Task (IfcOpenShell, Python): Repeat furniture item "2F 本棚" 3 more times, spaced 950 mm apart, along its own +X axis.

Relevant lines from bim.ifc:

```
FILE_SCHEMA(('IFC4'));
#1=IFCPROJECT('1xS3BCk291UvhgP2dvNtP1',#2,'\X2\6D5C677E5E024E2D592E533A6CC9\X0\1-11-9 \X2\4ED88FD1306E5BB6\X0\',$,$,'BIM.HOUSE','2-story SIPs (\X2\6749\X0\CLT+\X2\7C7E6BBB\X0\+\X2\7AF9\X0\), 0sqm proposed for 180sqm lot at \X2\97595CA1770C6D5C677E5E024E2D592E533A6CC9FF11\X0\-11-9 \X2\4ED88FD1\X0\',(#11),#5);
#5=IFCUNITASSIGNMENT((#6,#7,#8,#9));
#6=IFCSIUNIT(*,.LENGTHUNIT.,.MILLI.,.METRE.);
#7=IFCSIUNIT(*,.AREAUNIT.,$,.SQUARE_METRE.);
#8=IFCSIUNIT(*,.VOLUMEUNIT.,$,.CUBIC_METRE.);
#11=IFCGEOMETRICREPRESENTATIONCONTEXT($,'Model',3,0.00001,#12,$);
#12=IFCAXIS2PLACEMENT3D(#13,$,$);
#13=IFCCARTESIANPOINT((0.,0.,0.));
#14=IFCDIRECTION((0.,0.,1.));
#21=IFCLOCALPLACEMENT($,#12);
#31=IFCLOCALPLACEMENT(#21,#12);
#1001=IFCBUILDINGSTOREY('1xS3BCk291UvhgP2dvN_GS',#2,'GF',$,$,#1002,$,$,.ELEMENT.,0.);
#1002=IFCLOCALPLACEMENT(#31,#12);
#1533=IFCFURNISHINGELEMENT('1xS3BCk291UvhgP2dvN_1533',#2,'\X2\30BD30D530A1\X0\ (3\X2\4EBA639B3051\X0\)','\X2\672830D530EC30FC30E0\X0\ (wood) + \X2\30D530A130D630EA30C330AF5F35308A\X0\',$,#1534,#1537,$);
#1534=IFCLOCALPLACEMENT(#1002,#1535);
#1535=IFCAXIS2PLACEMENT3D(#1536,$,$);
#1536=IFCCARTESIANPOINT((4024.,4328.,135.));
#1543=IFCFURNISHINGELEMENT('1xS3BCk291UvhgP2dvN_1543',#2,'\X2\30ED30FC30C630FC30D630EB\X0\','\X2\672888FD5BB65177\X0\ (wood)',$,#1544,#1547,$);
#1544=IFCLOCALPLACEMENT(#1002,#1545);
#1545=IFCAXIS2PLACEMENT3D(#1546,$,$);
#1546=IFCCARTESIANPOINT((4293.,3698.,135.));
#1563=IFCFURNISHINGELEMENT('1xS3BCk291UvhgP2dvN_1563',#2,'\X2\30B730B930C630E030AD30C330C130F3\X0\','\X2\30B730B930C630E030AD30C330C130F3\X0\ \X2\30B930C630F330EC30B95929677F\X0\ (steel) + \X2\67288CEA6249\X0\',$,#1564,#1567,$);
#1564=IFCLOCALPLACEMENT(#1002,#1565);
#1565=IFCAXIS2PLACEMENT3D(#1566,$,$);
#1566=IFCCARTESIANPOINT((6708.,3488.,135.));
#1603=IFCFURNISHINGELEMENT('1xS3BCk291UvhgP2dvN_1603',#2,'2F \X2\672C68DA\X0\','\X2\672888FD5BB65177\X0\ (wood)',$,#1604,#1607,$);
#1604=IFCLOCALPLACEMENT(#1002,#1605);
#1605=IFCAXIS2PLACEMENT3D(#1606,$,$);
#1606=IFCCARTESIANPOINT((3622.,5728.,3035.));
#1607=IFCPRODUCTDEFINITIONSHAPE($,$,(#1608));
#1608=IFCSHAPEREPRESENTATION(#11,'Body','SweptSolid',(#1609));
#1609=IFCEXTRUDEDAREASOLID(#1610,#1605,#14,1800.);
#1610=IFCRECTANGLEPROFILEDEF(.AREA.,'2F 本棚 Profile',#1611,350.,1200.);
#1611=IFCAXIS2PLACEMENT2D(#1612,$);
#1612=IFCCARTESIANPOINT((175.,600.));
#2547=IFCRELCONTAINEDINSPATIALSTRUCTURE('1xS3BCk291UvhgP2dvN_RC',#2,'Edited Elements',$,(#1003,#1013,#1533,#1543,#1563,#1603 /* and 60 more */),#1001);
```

```python
import ifcopenshell
import ifcopenshell.api.geometry
import ifcopenshell.api.root
import ifcopenshell.util.element
import ifcopenshell.util.placement

model = ifcopenshell.open("bim.ifc")


def reuse_history(source, copy):
    """copy_class also copies each property set's owner history, people and application; keep the originals."""
    for rel in copy.IsDefinedBy:
        if rel.is_a("IfcRelDefinesByProperties") and (history := rel.RelatingPropertyDefinition.OwnerHistory):
            rel.RelatingPropertyDefinition.OwnerHistory = source.OwnerHistory
            ifcopenshell.util.element.remove_deep2(model, history)


source = model.by_guid("1xS3BCk291UvhgP2dvN_1603")
base = ifcopenshell.util.placement.get_local_placement(source.ObjectPlacement)
step = base[:3, 0] * 950.0

for i in range(1, 4):
    copy = ifcopenshell.api.root.copy_class(model, product=source)
    copy.Representation = ifcopenshell.util.element.copy_deep(
        model, source.Representation, exclude=["IfcGeometricRepresentationContext", "IfcRepresentationMap"]
    )
    reuse_history(source, copy)
    matrix = base.copy()
    matrix[:3, 3] += i * step
    print("added at", matrix[:3, 3].round(3) + 0.0)
    ifcopenshell.api.geometry.edit_object_placement(model, product=copy, matrix=matrix, is_si=False)

model.write("bim_rev.ifc")
```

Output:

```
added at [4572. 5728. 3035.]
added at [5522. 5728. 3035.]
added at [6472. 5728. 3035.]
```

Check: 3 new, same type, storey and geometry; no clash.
